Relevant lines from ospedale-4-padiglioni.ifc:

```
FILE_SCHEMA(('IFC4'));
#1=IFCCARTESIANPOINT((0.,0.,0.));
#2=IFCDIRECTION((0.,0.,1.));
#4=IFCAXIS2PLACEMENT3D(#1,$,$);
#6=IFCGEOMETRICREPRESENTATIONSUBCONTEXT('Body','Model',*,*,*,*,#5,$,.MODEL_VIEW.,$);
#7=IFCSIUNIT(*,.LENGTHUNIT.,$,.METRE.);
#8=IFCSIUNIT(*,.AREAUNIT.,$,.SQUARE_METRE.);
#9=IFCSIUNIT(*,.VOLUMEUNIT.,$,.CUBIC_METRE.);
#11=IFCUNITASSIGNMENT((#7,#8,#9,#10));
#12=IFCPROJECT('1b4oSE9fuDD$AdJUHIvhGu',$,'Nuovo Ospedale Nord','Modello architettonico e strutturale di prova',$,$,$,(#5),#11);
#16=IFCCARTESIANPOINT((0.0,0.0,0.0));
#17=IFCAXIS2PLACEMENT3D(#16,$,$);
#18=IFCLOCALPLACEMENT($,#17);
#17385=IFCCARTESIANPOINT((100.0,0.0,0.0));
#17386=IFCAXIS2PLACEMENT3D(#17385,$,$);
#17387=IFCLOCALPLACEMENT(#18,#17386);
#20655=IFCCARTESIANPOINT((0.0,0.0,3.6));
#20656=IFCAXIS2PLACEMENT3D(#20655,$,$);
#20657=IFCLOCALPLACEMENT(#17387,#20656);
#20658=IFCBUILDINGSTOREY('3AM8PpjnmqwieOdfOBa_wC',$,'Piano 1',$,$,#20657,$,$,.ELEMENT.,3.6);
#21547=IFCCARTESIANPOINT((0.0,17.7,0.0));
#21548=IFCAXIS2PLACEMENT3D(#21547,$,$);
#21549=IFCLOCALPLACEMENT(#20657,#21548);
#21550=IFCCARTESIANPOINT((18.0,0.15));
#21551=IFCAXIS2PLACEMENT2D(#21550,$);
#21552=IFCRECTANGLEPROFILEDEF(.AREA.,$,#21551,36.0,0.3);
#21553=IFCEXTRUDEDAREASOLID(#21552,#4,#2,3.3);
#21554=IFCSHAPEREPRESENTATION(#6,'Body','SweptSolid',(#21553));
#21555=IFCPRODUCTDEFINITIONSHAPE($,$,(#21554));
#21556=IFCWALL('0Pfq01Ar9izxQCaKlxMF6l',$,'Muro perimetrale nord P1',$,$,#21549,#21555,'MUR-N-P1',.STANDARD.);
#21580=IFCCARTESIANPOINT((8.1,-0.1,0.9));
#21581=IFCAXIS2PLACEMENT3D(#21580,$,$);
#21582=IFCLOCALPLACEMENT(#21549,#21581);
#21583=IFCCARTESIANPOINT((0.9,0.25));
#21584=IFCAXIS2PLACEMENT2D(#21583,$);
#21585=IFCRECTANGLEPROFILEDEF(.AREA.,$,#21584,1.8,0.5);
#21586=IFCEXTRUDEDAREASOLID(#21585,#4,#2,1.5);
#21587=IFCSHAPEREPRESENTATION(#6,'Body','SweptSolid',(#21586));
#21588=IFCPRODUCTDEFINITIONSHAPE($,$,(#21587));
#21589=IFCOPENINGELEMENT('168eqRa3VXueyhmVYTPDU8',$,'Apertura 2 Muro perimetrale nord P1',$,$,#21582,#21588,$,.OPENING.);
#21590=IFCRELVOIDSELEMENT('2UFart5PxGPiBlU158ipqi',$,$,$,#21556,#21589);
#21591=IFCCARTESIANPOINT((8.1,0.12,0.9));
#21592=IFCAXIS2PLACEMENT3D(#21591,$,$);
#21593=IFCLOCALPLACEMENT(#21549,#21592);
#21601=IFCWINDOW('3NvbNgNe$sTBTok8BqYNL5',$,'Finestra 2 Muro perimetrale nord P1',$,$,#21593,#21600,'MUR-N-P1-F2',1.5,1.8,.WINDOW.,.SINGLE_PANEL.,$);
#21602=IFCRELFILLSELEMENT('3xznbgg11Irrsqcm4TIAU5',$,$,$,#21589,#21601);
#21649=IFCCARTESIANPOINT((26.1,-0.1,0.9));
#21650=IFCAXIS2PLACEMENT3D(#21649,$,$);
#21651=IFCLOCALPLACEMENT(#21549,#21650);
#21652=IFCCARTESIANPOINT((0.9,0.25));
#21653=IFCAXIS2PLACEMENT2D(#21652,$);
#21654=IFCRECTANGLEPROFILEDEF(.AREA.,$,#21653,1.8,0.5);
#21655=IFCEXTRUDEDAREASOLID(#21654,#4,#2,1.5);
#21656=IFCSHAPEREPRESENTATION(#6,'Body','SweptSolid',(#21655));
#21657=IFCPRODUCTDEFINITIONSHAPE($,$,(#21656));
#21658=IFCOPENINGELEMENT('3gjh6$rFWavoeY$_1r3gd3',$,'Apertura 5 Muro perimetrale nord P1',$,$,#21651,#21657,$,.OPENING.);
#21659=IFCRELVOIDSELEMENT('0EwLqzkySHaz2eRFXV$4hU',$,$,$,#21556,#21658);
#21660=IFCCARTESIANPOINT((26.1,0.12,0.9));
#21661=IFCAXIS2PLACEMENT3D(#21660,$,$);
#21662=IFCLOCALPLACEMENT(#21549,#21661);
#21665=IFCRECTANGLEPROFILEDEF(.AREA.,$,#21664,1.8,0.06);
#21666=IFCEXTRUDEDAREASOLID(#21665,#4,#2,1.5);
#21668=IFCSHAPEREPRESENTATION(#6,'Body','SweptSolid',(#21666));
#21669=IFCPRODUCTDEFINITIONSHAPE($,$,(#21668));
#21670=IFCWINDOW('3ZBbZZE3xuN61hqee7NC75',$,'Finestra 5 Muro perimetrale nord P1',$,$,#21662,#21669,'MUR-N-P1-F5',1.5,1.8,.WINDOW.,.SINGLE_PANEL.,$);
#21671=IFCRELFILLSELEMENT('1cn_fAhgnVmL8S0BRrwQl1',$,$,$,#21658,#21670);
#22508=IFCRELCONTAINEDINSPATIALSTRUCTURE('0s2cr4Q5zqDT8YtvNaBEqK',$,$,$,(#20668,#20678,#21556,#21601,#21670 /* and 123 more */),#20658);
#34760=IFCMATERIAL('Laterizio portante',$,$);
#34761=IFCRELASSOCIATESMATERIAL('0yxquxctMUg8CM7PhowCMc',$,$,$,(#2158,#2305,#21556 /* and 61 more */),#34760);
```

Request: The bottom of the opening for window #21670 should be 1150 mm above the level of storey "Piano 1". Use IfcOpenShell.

```python
import numpy as np
import ifcopenshell
import ifcopenshell.api.geometry
import ifcopenshell.geom
import ifcopenshell.util.element
import ifcopenshell.util.placement
import ifcopenshell.util.shape
import ifcopenshell.util.unit

model = ifcopenshell.open("ospedale-4-padiglioni.ifc")
unit_scale = ifcopenshell.util.unit.calculate_unit_scale(model)

window = model.by_guid("3ZBbZZE3xuN61hqee7NC75")
opening = window.FillsVoids[0].RelatingOpeningElement
storey = ifcopenshell.util.element.get_container(window, ifc_class="IfcBuildingStorey")
level = ifcopenshell.util.placement.get_local_placement(storey.ObjectPlacement)[2, 3]

# The opening's origin need not be at the sill, so measure its lowest point.
shape = ifcopenshell.geom.create_shape(ifcopenshell.geom.settings(), opening)
bottom = ifcopenshell.util.shape.get_shape_bottom_elevation(shape, shape.geometry) / unit_scale
dz = level + 1.15 - bottom

shift = np.array([0.0, 0.0, dz])
# The window is not placed relative to its opening, so move both.
for product in (opening, window):
    matrix = ifcopenshell.util.placement.get_local_placement(product.ObjectPlacement)
    matrix[:3, 3] += shift
    ifcopenshell.api.geometry.edit_object_placement(model, product=product, matrix=matrix, is_si=False)

print(f"moved by {dz * unit_scale:+.3f} m")

model.write("ospedale-4-padiglioni_updated.ifc")
```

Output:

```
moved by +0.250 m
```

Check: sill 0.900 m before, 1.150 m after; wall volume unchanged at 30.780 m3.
